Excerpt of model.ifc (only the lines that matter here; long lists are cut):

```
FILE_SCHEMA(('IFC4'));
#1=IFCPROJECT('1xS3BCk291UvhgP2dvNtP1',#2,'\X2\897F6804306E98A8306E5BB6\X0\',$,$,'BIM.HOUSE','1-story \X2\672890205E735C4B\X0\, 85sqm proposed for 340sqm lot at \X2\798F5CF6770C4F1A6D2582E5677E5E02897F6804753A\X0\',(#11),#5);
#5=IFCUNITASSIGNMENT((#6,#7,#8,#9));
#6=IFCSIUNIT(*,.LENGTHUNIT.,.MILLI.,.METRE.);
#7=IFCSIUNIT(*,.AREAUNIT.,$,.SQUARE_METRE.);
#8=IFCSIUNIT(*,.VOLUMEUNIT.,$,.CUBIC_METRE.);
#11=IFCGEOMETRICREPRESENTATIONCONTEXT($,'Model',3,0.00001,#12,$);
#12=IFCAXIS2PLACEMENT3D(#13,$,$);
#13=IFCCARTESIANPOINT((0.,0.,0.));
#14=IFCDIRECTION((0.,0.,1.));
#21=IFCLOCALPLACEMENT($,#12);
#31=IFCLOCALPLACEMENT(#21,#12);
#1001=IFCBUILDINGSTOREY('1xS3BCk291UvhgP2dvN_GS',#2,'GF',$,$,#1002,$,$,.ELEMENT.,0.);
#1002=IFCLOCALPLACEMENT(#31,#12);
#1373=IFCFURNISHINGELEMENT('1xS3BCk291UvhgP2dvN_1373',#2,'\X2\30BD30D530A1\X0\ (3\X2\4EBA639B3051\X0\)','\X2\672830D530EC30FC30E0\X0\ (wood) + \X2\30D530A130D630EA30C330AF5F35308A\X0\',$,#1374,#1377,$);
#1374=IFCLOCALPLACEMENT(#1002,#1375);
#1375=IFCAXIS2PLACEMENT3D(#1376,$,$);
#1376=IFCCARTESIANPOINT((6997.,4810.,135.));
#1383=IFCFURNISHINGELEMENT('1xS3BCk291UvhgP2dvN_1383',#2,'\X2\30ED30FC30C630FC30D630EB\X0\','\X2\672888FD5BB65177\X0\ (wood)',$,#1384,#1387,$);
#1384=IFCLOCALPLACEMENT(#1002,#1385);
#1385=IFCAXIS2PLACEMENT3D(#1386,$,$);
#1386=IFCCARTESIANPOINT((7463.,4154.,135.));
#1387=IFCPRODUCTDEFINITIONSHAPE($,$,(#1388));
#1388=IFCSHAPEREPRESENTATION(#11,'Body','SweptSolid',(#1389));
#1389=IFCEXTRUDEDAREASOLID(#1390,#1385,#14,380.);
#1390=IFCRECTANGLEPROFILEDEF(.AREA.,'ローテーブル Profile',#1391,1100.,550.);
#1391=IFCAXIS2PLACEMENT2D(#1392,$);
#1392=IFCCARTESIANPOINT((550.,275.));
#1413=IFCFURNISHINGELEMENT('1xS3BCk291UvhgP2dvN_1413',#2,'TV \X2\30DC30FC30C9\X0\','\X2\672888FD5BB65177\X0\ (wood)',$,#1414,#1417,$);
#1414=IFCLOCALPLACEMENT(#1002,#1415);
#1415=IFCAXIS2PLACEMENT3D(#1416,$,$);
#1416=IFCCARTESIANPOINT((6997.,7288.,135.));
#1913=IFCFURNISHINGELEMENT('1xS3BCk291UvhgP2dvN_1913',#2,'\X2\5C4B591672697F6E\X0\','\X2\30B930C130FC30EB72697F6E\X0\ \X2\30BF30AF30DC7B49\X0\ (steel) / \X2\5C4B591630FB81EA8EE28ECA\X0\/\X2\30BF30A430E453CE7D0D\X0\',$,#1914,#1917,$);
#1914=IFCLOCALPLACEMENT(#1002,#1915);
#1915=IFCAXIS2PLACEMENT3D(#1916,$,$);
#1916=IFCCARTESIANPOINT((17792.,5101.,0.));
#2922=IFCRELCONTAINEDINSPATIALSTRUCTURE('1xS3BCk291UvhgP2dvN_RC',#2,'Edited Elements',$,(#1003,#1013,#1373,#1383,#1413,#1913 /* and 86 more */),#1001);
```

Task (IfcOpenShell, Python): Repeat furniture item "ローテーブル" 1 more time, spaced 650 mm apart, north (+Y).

```python
import numpy as np
import ifcopenshell
import ifcopenshell.api.geometry
import ifcopenshell.api.root
import ifcopenshell.util.element
import ifcopenshell.util.placement
import ifcopenshell.util.unit

model = ifcopenshell.open("model.ifc")
unit_scale = ifcopenshell.util.unit.calculate_unit_scale(model)


def reuse_history(source, copy):
    """copy_class also copies each property set's owner history, people and application; keep the originals."""
    for rel in copy.IsDefinedBy:
        if rel.is_a("IfcRelDefinesByProperties") and (history := rel.RelatingPropertyDefinition.OwnerHistory):
            rel.RelatingPropertyDefinition.OwnerHistory = source.OwnerHistory
            ifcopenshell.util.element.remove_deep2(model, history)


source = model.by_id(1383)
base = ifcopenshell.util.placement.get_local_placement(source.ObjectPlacement)
step = np.array([0.0, 1.0, 0.0]) * 0.65 / unit_scale

for i in range(1, 2):
    copy = ifcopenshell.api.root.copy_class(model, product=source)
    copy.Representation = ifcopenshell.util.element.copy_deep(
        model, source.Representation, exclude=["IfcGeometricRepresentationContext", "IfcRepresentationMap"]
    )
    reuse_history(source, copy)
    matrix = base.copy()
    matrix[:3, 3] += i * step
    print("added at", matrix[:3, 3].round(3) + 0.0)
    ifcopenshell.api.geometry.edit_object_placement(model, product=copy, matrix=matrix, is_si=False)

model.write("model_updated.ifc")
```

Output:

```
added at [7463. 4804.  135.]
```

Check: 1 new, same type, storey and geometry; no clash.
